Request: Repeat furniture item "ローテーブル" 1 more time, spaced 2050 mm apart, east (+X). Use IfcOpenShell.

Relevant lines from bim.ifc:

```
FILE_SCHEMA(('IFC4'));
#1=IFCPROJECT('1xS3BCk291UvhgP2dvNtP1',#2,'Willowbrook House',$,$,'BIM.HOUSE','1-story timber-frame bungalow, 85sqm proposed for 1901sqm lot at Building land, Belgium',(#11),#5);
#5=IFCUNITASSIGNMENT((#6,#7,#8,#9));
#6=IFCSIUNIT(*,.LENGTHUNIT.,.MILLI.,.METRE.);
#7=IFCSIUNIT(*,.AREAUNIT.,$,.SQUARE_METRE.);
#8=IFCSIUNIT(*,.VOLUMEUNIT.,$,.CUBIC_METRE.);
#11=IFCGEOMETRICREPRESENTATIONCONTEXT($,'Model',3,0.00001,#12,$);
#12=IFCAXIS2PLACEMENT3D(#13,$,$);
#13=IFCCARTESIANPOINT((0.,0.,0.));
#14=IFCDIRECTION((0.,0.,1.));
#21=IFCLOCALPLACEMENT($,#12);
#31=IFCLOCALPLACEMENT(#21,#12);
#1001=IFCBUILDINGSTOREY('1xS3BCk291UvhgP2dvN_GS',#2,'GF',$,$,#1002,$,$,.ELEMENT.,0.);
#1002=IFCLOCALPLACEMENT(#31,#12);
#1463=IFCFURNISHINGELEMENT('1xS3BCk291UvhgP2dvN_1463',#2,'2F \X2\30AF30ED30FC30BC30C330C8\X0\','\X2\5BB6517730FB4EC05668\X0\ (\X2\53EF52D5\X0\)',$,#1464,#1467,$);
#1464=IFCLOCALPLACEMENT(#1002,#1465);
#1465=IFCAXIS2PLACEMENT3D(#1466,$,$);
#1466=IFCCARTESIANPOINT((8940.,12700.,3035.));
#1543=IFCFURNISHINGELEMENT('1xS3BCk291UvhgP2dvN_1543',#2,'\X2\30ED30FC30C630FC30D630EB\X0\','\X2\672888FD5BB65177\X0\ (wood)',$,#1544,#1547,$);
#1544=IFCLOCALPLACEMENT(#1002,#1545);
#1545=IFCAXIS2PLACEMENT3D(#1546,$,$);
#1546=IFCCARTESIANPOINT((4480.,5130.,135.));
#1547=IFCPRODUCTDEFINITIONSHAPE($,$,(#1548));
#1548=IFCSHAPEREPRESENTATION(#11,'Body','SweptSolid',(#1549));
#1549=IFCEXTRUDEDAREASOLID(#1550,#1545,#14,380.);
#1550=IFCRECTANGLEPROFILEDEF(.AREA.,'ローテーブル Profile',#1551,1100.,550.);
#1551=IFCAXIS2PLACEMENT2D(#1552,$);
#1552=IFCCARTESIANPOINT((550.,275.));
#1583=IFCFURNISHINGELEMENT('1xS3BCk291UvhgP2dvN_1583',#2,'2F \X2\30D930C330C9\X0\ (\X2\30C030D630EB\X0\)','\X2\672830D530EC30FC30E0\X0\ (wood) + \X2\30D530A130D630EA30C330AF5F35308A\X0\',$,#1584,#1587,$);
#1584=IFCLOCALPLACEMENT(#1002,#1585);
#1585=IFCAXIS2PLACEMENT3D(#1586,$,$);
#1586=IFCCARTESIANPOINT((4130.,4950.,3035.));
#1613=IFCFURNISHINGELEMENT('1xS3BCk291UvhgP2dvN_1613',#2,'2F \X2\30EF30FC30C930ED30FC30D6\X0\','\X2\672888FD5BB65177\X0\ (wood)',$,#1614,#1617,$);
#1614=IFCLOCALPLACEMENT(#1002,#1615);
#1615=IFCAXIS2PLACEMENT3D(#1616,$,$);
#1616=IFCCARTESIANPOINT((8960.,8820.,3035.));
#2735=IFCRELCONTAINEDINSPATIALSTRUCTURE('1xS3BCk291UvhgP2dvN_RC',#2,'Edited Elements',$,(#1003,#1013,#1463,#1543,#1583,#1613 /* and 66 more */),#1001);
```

```python
import numpy as np
import ifcopenshell
import ifcopenshell.api.geometry
import ifcopenshell.api.root
import ifcopenshell.util.element
import ifcopenshell.util.placement

model = ifcopenshell.open("bim.ifc")


def reuse_history(source, copy):
    """copy_class also copies each property set's owner history, people and application; keep the originals."""
    for rel in copy.IsDefinedBy:
        if rel.is_a("IfcRelDefinesByProperties") and (history := rel.RelatingPropertyDefinition.OwnerHistory):
            rel.RelatingPropertyDefinition.OwnerHistory = source.OwnerHistory
            ifcopenshell.util.element.remove_deep2(model, history)


source = model.by_id(1543)
base = ifcopenshell.util.placement.get_local_placement(source.ObjectPlacement)
step = np.array([1.0, 0.0, 0.0]) * 2050.0

for i in range(1, 2):
    copy = ifcopenshell.api.root.copy_class(model, product=source)
    copy.Representation = ifcopenshell.util.element.copy_deep(
        model, source.Representation, exclude=["IfcGeometricRepresentationContext", "IfcRepresentationMap"]
    )
    reuse_history(source, copy)
    matrix = base.copy()
    matrix[:3, 3] += i * step
    print("added at", matrix[:3, 3].round(3) + 0.0)
    ifcopenshell.api.geometry.edit_object_placement(model, product=copy, matrix=matrix, is_si=False)

model.write("bim-out.ifc")
```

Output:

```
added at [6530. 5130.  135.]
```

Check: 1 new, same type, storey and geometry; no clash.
